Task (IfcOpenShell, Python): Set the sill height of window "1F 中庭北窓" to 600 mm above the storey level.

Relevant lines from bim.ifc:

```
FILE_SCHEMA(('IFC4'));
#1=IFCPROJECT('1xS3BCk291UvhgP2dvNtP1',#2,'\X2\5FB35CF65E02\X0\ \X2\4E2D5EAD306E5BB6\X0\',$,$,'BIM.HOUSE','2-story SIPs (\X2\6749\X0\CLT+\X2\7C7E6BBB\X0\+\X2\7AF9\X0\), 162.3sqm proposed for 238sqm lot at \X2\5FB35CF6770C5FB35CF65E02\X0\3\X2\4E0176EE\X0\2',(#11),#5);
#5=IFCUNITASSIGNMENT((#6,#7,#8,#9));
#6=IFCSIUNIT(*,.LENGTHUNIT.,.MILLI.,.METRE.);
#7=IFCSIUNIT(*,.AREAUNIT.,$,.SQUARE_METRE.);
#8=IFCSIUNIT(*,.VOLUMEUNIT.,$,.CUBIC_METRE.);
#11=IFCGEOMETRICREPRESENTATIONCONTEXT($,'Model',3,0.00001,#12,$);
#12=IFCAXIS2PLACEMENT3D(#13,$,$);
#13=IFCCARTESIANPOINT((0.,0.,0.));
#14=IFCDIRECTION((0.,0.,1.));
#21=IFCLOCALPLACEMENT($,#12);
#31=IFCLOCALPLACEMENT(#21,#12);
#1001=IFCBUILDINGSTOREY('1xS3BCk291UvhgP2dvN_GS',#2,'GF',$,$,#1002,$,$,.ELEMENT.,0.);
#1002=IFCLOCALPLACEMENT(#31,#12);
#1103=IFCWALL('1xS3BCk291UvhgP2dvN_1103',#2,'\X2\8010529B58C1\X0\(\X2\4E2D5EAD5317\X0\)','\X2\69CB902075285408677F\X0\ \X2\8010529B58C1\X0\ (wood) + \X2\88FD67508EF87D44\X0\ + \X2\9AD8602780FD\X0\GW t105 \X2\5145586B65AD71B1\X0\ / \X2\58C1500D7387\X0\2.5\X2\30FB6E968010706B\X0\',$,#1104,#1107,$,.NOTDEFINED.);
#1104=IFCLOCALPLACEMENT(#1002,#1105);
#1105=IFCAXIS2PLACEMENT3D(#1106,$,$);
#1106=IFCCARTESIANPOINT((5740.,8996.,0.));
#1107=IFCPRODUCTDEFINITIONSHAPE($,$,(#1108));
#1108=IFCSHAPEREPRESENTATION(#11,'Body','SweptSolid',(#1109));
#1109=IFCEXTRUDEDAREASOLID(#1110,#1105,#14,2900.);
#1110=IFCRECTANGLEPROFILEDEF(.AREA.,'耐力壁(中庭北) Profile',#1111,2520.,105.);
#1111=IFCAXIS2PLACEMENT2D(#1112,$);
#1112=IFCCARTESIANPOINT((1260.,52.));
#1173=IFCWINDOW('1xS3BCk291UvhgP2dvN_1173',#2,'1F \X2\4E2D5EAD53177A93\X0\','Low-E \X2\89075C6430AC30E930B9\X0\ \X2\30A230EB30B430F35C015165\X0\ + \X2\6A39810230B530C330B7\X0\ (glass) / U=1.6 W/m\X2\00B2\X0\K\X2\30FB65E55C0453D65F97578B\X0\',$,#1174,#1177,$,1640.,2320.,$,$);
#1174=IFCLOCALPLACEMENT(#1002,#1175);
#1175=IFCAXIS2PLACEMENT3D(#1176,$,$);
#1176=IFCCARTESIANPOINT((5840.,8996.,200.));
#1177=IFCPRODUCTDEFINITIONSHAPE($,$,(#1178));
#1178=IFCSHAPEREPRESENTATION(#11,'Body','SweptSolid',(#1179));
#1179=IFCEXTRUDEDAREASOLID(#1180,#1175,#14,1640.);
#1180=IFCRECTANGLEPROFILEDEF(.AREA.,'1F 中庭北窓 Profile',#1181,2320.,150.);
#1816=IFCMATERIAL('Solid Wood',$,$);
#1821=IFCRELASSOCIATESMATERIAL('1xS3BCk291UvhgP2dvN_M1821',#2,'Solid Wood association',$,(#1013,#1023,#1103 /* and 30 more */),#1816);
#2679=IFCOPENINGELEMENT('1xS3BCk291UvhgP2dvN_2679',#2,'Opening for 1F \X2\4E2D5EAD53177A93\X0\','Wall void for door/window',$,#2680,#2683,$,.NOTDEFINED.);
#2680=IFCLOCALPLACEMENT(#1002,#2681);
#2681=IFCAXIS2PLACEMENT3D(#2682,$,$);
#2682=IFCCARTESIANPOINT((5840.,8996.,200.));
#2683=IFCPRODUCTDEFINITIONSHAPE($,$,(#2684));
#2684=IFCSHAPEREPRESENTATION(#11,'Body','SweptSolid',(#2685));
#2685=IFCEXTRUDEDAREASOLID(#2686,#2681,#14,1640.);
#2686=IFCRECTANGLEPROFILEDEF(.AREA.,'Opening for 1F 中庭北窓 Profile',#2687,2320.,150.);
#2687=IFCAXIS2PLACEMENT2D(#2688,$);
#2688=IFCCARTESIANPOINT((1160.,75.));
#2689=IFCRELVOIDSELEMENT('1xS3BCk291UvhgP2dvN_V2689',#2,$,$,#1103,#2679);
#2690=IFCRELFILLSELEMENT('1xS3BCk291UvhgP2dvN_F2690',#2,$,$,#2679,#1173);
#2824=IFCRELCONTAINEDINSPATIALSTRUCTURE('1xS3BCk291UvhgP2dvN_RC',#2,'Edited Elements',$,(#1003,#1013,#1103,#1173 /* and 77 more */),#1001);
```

```python
import numpy as np
import ifcopenshell
import ifcopenshell.api.geometry
import ifcopenshell.geom
import ifcopenshell.util.element
import ifcopenshell.util.placement
import ifcopenshell.util.shape
import ifcopenshell.util.unit

model = ifcopenshell.open("bim.ifc")
unit_scale = ifcopenshell.util.unit.calculate_unit_scale(model)

window = model.by_guid("1xS3BCk291UvhgP2dvN_1173")
opening = window.FillsVoids[0].RelatingOpeningElement
storey = ifcopenshell.util.element.get_container(window, ifc_class="IfcBuildingStorey")
level = ifcopenshell.util.placement.get_local_placement(storey.ObjectPlacement)[2, 3]

# The opening's origin need not be at the sill, so measure its lowest point.
shape = ifcopenshell.geom.create_shape(ifcopenshell.geom.settings(), opening)
bottom = ifcopenshell.util.shape.get_shape_bottom_elevation(shape, shape.geometry) / unit_scale
dz = level + 0.6 / unit_scale - bottom

shift = np.array([0.0, 0.0, dz])
# The window is not placed relative to its opening, so move both.
for product in (opening, window):
    matrix = ifcopenshell.util.placement.get_local_placement(product.ObjectPlacement)
    matrix[:3, 3] += shift
    ifcopenshell.api.geometry.edit_object_placement(model, product=product, matrix=matrix, is_si=False)

print(f"moved by {dz * unit_scale:+.3f} m")

model.write("bim_updated.ifc")
```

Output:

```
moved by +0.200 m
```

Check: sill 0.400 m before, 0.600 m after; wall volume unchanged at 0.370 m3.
